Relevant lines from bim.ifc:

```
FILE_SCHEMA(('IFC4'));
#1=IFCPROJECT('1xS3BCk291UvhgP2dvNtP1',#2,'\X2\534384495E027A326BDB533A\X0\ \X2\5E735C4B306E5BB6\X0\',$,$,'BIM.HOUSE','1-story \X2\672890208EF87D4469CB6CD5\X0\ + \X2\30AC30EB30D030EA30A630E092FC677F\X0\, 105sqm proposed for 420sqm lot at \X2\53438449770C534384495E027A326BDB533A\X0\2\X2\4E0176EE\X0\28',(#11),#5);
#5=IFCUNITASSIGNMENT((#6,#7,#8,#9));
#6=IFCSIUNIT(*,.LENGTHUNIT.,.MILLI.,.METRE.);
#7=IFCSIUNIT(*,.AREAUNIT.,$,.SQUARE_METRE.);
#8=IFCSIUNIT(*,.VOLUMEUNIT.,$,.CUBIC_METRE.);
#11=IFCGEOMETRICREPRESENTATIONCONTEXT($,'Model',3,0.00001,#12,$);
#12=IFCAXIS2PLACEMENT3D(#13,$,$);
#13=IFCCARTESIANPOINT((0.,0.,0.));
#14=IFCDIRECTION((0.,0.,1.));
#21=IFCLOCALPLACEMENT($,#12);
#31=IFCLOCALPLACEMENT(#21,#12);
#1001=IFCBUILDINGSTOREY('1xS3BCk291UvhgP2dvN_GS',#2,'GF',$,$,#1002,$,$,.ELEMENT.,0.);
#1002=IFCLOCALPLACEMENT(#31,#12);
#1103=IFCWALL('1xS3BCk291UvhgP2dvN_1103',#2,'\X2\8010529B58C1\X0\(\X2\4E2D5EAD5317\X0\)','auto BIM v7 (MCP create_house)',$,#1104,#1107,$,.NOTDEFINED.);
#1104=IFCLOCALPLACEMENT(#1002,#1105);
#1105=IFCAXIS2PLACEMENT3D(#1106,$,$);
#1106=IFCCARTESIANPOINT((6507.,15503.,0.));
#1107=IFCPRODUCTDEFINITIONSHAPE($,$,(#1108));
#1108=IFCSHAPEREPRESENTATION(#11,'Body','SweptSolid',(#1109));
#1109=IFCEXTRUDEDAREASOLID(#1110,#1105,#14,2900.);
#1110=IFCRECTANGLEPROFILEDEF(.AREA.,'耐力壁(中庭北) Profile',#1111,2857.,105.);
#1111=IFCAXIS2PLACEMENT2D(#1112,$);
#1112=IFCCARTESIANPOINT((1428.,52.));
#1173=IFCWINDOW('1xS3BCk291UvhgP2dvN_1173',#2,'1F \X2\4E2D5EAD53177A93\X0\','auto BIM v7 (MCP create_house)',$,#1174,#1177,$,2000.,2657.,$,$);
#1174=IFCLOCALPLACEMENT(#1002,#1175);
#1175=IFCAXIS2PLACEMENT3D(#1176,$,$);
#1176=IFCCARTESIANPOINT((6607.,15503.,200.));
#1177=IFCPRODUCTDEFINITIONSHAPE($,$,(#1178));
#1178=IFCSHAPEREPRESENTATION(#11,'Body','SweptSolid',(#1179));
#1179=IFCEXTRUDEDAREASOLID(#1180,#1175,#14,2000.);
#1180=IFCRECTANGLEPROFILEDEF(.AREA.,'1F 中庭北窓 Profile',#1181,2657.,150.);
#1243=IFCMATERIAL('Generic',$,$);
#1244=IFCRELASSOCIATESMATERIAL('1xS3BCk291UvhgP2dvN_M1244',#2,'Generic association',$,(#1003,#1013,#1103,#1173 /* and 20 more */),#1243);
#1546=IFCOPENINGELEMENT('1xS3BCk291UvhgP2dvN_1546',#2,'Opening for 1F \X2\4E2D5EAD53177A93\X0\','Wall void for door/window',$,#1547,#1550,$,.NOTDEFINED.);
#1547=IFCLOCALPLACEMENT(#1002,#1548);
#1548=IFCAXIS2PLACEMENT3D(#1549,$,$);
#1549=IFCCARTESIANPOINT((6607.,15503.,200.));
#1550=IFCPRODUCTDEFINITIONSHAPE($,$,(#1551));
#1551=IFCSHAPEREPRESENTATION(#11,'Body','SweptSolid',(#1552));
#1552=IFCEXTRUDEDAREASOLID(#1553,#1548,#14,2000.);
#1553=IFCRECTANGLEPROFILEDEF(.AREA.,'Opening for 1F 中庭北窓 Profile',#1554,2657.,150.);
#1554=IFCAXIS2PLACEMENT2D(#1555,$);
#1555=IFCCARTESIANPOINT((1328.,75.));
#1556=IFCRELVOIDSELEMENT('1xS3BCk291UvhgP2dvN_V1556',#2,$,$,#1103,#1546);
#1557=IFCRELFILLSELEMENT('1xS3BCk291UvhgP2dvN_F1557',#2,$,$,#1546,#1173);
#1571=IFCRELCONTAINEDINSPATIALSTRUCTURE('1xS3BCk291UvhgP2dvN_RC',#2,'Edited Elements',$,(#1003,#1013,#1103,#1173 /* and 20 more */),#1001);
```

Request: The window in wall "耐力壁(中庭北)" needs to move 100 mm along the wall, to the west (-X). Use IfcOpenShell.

```python
import ifcopenshell
import ifcopenshell.api.geometry
import ifcopenshell.util.placement
import ifcopenshell.util.unit

model = ifcopenshell.open("bim.ifc")
unit_scale = ifcopenshell.util.unit.calculate_unit_scale(model)

window = model.by_guid("1xS3BCk291UvhgP2dvN_1173")
opening = window.FillsVoids[0].RelatingOpeningElement
wall = opening.VoidsElements[0].RelatingBuildingElement

wall_matrix = ifcopenshell.util.placement.get_local_placement(wall.ObjectPlacement)
shift = wall_matrix[:3, 0] * -0.1 / unit_scale
before = ifcopenshell.util.placement.get_local_placement(window.ObjectPlacement)[:3, 3].copy()

# The window is not placed relative to its opening, so move both.
for product in (opening, window):
    matrix = ifcopenshell.util.placement.get_local_placement(product.ObjectPlacement)
    matrix[:3, 3] += shift
    ifcopenshell.api.geometry.edit_object_placement(model, product=product, matrix=matrix, is_si=False)

after = ifcopenshell.util.placement.get_local_placement(window.ObjectPlacement)[:3, 3]
print("window moved by", (after - before).round(3) + 0.0)

model.write("bim_v2.ifc")
```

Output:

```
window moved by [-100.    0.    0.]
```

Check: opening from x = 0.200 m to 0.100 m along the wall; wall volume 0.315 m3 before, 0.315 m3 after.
